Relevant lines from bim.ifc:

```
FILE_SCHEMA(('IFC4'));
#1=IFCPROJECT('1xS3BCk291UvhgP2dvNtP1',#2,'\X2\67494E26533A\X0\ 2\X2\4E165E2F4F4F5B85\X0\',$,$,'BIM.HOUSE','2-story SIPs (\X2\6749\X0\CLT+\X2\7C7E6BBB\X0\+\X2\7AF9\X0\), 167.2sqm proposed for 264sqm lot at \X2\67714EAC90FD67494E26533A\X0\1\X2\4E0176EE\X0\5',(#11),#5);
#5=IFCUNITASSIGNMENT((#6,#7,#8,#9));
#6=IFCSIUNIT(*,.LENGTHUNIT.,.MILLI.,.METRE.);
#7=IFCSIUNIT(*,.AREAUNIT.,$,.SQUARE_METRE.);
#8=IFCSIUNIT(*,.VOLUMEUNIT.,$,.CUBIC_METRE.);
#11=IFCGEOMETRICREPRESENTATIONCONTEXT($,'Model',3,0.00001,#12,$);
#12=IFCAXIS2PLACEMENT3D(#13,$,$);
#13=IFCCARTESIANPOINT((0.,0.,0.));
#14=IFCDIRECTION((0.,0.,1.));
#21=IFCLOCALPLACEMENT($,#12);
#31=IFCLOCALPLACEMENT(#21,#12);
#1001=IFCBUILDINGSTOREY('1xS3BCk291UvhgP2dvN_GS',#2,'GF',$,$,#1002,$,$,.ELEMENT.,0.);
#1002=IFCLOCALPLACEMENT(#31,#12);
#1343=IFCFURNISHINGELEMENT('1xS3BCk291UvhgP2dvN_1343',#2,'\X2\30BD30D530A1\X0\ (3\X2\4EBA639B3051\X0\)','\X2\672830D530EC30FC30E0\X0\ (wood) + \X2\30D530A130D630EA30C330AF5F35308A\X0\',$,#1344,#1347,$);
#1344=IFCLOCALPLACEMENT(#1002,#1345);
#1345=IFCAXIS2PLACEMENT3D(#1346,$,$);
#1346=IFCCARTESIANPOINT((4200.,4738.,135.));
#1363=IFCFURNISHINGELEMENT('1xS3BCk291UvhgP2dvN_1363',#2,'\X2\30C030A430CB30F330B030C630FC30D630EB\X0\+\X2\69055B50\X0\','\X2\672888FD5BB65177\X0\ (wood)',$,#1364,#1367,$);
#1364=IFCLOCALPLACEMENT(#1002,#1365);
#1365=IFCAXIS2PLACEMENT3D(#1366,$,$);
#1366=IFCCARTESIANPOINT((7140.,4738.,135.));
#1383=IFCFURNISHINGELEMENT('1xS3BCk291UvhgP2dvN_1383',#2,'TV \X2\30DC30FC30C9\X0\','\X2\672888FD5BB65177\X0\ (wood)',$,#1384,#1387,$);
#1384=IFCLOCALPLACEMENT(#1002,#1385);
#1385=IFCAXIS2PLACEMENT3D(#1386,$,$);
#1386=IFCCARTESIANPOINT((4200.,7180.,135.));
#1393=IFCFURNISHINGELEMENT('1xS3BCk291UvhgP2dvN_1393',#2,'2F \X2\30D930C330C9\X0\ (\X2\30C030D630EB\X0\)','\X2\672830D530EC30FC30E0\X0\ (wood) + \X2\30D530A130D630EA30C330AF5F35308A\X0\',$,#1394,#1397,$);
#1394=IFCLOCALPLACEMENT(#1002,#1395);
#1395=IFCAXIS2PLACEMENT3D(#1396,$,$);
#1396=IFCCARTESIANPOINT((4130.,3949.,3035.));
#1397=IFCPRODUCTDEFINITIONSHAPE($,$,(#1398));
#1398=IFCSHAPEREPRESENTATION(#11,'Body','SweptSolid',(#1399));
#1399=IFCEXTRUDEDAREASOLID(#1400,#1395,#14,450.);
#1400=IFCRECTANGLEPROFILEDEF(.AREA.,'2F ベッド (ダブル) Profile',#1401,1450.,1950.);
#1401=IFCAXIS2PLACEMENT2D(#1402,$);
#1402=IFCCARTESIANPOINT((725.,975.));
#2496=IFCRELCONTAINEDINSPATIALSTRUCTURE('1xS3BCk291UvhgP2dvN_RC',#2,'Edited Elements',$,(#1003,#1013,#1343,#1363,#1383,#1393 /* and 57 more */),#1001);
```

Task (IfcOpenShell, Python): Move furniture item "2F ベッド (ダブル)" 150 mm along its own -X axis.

```python
import ifcopenshell
import ifcopenshell.api.geometry
import ifcopenshell.util.placement

model = ifcopenshell.open("bim.ifc")

item = model.by_guid("1xS3BCk291UvhgP2dvN_1393")
matrix = ifcopenshell.util.placement.get_local_placement(item.ObjectPlacement)
matrix[:3, 3] -= matrix[:3, 0] * 150.0
ifcopenshell.api.geometry.edit_object_placement(model, product=item, matrix=matrix, is_si=False)

print(ifcopenshell.util.placement.get_local_placement(item.ObjectPlacement).round(3) + 0.0)

model.write("bim-out.ifc")
```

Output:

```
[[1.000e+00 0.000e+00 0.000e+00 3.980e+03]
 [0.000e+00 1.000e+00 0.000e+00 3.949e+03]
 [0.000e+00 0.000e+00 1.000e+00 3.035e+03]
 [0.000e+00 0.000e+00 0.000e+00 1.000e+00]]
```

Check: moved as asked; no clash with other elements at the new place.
